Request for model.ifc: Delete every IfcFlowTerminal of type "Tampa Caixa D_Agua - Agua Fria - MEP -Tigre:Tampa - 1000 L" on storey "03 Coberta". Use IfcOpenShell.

First a look at what the model holds.

```python
import ifcopenshell
import ifcopenshell.util.element

model = ifcopenshell.open("model.ifc")
print(model.schema)
storey = next(s for s in model.by_type("IfcBuildingStorey") if s.Name == "03 Coberta")
terminals = [e for e in ifcopenshell.util.element.get_decomposition(storey) if e.is_a("IfcFlowTerminal")]
seen = {}
for e in terminals:
    element_type = ifcopenshell.util.element.get_type(e)
    name = element_type.Name if element_type not in (None, e) else None
    seen[name] = seen.get(name, 0) + 1
for name, count in sorted(seen.items(), key=str):
    print(count, "x", name)
```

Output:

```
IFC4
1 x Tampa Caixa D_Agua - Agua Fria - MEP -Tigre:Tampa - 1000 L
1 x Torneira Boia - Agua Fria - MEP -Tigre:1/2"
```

```python
import ifcopenshell
import ifcopenshell.api.root
import ifcopenshell.util.element

model = ifcopenshell.open("model.ifc")

storey = next(s for s in model.by_type("IfcBuildingStorey") if s.Name == "03 Coberta")
terminals = [e for e in ifcopenshell.util.element.get_decomposition(storey) if e.is_a("IfcFlowTerminal")]
targets = [e for e in terminals if (t := ifcopenshell.util.element.get_type(e)) not in (None, e) and t.Name == "Tampa Caixa D_Agua - Agua Fria - MEP -Tigre:Tampa - 1000 L"]

for e in targets:
    ifcopenshell.api.root.remove_product(model, product=e)
print(len(targets), "removed")

model.write("model_edited.ifc")
```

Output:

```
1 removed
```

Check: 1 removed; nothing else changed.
